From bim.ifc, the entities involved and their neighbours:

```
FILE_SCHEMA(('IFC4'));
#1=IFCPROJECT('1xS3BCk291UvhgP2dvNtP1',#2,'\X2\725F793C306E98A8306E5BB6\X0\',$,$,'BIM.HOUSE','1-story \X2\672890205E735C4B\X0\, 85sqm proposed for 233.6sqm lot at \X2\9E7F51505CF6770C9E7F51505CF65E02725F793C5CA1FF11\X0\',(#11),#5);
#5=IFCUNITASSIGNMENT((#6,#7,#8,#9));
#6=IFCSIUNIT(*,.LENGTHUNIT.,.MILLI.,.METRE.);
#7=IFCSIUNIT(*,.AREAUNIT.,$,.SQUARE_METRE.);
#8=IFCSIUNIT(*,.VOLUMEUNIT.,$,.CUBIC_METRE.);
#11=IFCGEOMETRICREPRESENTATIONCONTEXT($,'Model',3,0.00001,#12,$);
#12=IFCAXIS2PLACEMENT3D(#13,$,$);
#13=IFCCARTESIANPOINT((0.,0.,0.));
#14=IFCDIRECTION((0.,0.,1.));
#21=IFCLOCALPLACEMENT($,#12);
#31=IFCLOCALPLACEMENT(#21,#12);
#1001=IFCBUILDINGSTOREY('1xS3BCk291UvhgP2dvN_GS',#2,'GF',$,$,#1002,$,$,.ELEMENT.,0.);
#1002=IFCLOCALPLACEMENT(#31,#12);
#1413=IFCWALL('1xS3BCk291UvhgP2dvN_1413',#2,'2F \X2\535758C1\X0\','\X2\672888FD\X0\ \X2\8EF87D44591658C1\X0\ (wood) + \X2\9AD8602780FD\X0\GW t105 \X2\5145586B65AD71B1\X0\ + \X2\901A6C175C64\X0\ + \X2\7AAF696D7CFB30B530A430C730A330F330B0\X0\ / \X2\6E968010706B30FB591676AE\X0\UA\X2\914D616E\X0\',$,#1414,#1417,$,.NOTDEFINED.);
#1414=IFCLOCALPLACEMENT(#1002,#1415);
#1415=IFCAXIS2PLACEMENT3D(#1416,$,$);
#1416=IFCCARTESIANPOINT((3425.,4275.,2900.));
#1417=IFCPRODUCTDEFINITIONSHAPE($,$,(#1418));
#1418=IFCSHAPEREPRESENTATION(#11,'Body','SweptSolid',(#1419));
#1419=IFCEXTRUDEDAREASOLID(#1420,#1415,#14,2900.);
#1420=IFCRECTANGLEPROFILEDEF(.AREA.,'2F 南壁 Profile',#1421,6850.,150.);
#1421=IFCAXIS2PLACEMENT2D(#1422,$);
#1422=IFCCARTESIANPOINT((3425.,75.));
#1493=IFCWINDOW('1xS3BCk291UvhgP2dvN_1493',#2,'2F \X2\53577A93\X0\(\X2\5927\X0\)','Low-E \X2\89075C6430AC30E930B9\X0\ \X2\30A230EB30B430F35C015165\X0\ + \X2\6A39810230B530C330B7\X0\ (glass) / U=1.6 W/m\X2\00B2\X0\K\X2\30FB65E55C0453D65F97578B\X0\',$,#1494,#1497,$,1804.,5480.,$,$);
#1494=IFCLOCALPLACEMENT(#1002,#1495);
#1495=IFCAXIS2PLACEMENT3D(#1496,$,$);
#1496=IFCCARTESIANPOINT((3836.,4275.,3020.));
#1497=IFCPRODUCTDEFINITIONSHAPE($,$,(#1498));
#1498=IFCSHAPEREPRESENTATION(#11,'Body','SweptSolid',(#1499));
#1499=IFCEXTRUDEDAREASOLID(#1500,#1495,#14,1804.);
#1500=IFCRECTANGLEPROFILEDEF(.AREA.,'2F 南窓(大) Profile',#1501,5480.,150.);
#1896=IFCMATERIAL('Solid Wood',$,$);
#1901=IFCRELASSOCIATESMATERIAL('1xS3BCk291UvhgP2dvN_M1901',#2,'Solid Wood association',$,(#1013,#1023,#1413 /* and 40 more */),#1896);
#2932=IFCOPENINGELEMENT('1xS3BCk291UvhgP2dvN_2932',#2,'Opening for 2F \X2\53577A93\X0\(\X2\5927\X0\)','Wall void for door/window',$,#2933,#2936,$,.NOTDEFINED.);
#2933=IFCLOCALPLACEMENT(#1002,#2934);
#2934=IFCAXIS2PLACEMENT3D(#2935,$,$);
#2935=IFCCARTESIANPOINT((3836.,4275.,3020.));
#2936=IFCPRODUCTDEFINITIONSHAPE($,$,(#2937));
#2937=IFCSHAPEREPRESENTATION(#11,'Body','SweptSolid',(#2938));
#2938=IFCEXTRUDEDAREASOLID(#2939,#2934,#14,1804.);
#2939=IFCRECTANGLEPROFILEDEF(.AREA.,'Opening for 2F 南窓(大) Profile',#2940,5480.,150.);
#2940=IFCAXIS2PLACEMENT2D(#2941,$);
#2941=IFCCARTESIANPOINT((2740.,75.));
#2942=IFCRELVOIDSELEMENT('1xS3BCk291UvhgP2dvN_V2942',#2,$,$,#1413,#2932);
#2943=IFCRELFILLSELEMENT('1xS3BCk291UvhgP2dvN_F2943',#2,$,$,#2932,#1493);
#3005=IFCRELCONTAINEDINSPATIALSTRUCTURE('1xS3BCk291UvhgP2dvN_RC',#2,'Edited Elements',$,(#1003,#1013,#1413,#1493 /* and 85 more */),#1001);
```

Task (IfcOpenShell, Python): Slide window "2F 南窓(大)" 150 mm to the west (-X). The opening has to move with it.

```python
import ifcopenshell
import ifcopenshell.api.geometry
import ifcopenshell.util.placement
import ifcopenshell.util.unit

model = ifcopenshell.open("bim.ifc")
unit_scale = ifcopenshell.util.unit.calculate_unit_scale(model)

window = model.by_guid("1xS3BCk291UvhgP2dvN_1493")
opening = window.FillsVoids[0].RelatingOpeningElement
wall = opening.VoidsElements[0].RelatingBuildingElement

wall_matrix = ifcopenshell.util.placement.get_local_placement(wall.ObjectPlacement)
shift = wall_matrix[:3, 0] * -0.15 / unit_scale
before = ifcopenshell.util.placement.get_local_placement(window.ObjectPlacement)[:3, 3].copy()

# The window is not placed relative to its opening, so move both.
for product in (opening, window):
    matrix = ifcopenshell.util.placement.get_local_placement(product.ObjectPlacement)
    matrix[:3, 3] += shift
    ifcopenshell.api.geometry.edit_object_placement(model, product=product, matrix=matrix, is_si=False)

after = ifcopenshell.util.placement.get_local_placement(window.ObjectPlacement)[:3, 3]
print("window moved by", (after - before).round(3) + 0.0)

model.write("bim_v2.ifc")
```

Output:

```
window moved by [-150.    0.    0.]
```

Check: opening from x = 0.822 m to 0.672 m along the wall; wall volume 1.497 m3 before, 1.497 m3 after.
